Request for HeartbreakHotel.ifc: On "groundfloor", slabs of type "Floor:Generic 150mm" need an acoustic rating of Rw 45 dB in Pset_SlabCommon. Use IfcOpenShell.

First a look at what the model holds.

```python
import ifcopenshell
import ifcopenshell.util.element

model = ifcopenshell.open("HeartbreakHotel.ifc")
print(model.schema)
storey = next(s for s in model.by_type("IfcBuildingStorey") if s.Name == "groundfloor")
slabs = [e for e in ifcopenshell.util.element.get_decomposition(storey) if e.is_a("IfcSlab")]
seen = {}
for e in slabs:
    element_type = ifcopenshell.util.element.get_type(e)
    key = (element_type.Name if element_type != e and element_type else None, ifcopenshell.util.element.get_pset(e, "Pset_SlabCommon", "AcousticRating"))
    seen[key] = seen.get(key, 0) + 1
for (name, value), count in sorted(seen.items(), key=str):
    print(count, "x", name, "|", value)
```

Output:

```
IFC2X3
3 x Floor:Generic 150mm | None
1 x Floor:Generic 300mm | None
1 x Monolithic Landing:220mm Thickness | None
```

```python
import ifcopenshell
import ifcopenshell.api.pset
import ifcopenshell.util.element

model = ifcopenshell.open("HeartbreakHotel.ifc")

storey = next(s for s in model.by_type("IfcBuildingStorey") if s.Name == "groundfloor")
slabs = [e for e in ifcopenshell.util.element.get_decomposition(storey) if e.is_a("IfcSlab")]

count = 0
for e in slabs:
    element_type = ifcopenshell.util.element.get_type(e)
    if element_type in (None, e) or element_type.Name != "Floor:Generic 150mm":
        continue
    # add_pset returns the element's existing set when there is one.
    pset = ifcopenshell.api.pset.add_pset(model, product=e, name="Pset_SlabCommon")
    ifcopenshell.api.pset.edit_pset(model, pset=pset, properties={"AcousticRating": "Rw 45 dB"})
    count += 1

print(count, "slabs updated")

model.write("HeartbreakHotel-out.ifc")
```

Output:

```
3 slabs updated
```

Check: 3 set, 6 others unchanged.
